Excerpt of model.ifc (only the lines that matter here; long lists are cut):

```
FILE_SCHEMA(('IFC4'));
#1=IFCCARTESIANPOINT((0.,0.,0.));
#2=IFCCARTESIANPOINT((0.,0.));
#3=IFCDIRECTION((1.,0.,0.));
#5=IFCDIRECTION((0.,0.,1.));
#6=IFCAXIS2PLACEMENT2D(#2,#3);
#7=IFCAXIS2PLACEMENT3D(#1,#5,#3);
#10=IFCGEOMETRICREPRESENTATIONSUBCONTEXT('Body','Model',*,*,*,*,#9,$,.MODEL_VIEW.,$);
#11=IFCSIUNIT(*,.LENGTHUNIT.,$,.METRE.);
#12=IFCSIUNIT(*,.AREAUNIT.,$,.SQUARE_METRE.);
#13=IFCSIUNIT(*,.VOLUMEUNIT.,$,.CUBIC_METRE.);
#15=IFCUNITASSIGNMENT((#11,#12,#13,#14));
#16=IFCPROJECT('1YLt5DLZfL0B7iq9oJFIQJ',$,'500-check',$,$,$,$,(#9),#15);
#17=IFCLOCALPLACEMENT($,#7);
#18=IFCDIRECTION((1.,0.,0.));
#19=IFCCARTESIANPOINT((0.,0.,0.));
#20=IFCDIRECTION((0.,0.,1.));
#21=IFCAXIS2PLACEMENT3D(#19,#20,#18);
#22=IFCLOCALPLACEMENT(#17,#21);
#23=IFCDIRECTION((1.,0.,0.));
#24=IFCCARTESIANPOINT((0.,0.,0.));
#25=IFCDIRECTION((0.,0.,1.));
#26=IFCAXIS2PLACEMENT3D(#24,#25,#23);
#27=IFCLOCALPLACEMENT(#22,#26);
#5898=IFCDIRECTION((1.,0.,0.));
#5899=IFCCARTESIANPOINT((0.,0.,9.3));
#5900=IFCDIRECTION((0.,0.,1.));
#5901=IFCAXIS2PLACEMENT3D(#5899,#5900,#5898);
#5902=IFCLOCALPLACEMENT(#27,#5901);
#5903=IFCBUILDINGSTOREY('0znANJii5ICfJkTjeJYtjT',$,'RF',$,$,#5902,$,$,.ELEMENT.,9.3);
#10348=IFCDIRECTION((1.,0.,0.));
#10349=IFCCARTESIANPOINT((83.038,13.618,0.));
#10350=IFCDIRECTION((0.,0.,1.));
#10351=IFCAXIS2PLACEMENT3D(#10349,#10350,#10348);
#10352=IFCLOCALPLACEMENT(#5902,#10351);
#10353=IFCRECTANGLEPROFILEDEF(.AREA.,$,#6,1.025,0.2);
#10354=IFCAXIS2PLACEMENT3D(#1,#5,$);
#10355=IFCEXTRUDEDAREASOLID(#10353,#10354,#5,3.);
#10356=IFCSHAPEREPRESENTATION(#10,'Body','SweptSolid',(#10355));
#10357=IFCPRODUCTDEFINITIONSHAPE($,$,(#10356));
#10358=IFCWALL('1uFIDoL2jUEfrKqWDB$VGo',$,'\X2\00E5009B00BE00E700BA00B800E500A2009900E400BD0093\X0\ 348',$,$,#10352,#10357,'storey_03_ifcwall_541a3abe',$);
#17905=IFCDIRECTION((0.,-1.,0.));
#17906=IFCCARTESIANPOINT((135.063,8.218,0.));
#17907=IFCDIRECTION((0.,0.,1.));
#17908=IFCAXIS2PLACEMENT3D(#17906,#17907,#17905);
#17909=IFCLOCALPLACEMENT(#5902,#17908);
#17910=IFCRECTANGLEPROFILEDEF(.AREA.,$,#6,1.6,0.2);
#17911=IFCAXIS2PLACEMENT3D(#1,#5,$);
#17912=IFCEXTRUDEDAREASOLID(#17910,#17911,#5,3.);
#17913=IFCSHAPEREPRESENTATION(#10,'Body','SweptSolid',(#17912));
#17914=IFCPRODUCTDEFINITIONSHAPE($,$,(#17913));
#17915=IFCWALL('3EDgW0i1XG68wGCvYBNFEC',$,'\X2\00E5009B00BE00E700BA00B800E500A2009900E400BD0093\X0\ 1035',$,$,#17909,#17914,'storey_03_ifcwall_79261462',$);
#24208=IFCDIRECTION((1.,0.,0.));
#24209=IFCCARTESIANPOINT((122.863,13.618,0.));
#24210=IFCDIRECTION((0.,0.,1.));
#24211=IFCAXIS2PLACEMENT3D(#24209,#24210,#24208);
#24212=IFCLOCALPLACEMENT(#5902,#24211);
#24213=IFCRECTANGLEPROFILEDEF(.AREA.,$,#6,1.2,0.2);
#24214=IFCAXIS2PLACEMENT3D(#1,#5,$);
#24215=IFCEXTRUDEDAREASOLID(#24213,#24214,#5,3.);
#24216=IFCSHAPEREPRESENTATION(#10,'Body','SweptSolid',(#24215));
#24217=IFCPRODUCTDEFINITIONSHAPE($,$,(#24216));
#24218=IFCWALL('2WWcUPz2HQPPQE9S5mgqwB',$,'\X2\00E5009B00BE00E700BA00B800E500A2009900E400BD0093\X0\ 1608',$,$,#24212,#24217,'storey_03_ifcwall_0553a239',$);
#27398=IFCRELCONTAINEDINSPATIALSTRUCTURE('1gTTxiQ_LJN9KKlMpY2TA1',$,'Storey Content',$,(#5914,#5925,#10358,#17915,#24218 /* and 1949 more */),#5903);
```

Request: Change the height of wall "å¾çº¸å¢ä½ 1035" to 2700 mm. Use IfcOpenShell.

```python
import ifcopenshell
import ifcopenshell.geom
import ifcopenshell.util.representation
import ifcopenshell.util.shape
import ifcopenshell.util.unit

model = ifcopenshell.open("model.ifc")
unit_scale = ifcopenshell.util.unit.calculate_unit_scale(model)
settings = ifcopenshell.geom.settings()


def volume(element):
    """Net volume in cubic metres, openings subtracted."""
    shape = ifcopenshell.geom.create_shape(settings, element)
    return ifcopenshell.util.shape.get_volume(shape.geometry)


wall = model.by_guid("3EDgW0i1XG68wGCvYBNFEC")
before = volume(wall)

body = ifcopenshell.util.representation.get_representation(wall, "Model", "Body")
solid = body.Items[0]
old_height = solid.Depth
solid.Depth = 2.7 / unit_scale
after = volume(wall)

print(f"height {old_height:g} -> {solid.Depth:g}, volume {before:.3f} -> {after:.3f} m3")

model.write("model_rev.ifc")
```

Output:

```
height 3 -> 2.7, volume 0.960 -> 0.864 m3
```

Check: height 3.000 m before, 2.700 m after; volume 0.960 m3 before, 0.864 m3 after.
